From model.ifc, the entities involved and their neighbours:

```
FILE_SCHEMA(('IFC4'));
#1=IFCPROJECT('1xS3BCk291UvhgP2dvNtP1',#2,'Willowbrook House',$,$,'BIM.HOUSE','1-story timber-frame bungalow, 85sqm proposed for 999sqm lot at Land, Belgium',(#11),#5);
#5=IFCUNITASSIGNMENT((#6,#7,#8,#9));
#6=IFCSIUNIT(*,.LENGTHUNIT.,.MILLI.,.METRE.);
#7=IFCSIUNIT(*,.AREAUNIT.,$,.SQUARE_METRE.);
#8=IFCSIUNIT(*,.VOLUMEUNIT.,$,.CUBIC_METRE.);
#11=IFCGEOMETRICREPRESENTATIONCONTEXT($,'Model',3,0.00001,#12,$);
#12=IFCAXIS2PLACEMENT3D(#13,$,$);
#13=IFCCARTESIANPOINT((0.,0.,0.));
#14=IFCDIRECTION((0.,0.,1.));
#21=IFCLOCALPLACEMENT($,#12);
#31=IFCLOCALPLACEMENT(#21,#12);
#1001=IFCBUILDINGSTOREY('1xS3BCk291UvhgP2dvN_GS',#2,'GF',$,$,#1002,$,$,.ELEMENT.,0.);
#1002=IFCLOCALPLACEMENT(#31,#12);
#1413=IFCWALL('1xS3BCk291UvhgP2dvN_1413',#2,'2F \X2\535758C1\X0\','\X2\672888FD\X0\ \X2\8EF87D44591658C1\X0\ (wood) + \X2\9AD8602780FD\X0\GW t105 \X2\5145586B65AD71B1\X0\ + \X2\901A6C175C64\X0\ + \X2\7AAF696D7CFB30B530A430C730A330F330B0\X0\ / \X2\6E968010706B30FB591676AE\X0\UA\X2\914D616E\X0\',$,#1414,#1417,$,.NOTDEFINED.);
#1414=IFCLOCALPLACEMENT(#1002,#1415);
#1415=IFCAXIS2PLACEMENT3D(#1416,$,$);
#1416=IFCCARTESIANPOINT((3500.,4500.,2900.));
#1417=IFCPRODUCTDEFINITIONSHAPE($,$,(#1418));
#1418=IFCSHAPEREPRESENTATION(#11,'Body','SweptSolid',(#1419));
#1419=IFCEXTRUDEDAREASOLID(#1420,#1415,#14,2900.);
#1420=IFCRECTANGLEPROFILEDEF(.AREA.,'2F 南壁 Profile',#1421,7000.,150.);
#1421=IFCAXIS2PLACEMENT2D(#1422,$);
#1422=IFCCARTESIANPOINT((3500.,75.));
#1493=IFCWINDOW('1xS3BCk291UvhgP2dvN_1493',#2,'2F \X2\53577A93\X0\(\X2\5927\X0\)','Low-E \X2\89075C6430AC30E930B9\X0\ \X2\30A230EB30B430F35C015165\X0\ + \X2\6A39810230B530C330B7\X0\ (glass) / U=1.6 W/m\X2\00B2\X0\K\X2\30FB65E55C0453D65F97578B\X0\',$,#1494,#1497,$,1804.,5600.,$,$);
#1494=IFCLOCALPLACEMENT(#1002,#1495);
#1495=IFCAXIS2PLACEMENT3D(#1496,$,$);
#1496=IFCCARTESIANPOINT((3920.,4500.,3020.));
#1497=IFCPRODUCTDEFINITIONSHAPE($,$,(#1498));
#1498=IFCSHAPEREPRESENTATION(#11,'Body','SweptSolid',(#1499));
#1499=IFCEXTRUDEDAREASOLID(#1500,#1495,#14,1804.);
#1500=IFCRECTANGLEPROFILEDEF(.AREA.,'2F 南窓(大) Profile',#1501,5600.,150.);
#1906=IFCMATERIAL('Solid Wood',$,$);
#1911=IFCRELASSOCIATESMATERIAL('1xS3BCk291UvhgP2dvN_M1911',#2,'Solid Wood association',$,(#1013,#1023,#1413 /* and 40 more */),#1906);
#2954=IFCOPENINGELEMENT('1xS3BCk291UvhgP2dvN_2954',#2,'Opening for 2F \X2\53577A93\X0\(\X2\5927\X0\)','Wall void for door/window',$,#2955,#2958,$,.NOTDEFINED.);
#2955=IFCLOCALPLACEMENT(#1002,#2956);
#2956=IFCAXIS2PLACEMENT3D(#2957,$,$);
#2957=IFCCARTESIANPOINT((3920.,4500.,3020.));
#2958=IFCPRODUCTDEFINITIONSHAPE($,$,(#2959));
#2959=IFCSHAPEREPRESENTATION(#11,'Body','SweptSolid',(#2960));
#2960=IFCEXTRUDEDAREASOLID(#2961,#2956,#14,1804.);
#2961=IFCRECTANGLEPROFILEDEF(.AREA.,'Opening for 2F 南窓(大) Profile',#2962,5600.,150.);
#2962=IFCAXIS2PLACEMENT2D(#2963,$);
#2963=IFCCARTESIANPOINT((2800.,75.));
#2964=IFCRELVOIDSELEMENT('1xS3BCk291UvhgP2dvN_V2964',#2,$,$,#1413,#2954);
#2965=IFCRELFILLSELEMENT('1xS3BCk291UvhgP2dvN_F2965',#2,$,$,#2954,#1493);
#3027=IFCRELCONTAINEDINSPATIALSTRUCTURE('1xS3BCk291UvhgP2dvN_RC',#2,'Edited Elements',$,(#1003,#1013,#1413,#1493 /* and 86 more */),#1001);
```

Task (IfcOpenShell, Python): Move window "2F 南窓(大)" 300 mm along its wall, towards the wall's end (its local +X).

```python
import ifcopenshell
import ifcopenshell.api.geometry
import ifcopenshell.util.placement
import ifcopenshell.util.unit

model = ifcopenshell.open("model.ifc")
unit_scale = ifcopenshell.util.unit.calculate_unit_scale(model)

window = model.by_guid("1xS3BCk291UvhgP2dvN_1493")
opening = window.FillsVoids[0].RelatingOpeningElement
wall = opening.VoidsElements[0].RelatingBuildingElement

wall_matrix = ifcopenshell.util.placement.get_local_placement(wall.ObjectPlacement)
shift = wall_matrix[:3, 0] * 0.3 / unit_scale
before = ifcopenshell.util.placement.get_local_placement(window.ObjectPlacement)[:3, 3].copy()

# The window is not placed relative to its opening, so move both.
for product in (opening, window):
    matrix = ifcopenshell.util.placement.get_local_placement(product.ObjectPlacement)
    matrix[:3, 3] += shift
    ifcopenshell.api.geometry.edit_object_placement(model, product=product, matrix=matrix, is_si=False)

after = ifcopenshell.util.placement.get_local_placement(window.ObjectPlacement)[:3, 3]
print("window moved by", (after - before).round(3) + 0.0)

model.write("model-out.ifc")
```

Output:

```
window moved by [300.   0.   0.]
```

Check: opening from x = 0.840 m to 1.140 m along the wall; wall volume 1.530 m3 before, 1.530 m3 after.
